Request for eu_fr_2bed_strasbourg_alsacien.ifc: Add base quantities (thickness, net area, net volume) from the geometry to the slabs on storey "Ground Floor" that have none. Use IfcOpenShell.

First a look at what the model holds.

```python
import ifcopenshell
import ifcopenshell.util.element
import ifcopenshell.util.unit

model = ifcopenshell.open("eu_fr_2bed_strasbourg_alsacien.ifc")
print(model.schema)
for unit_type in ("LENGTHUNIT", "AREAUNIT", "VOLUMEUNIT"):
    print(unit_type, ifcopenshell.util.unit.calculate_unit_scale(model, unit_type))
storey = next(s for s in model.by_type("IfcBuildingStorey") if s.Name == "Ground Floor")
slabs = [e for e in ifcopenshell.util.element.get_decomposition(storey) if e.is_a("IfcSlab")]
for e in sorted(slabs, key=lambda e: e.id()):
    print(e.id(), e.is_a(), e.Name, list(ifcopenshell.util.element.get_psets(e, qtos_only=True)), sep=" | ")
```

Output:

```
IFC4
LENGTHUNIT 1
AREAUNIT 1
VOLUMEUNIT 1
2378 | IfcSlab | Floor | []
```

```python
import ifcopenshell
import ifcopenshell.api.pset
import ifcopenshell.geom
import ifcopenshell.util.element
import ifcopenshell.util.shape
import ifcopenshell.util.unit

model = ifcopenshell.open("eu_fr_2bed_strasbourg_alsacien.ifc")
unit_scale = ifcopenshell.util.unit.calculate_unit_scale(model)
area_scale = ifcopenshell.util.unit.calculate_unit_scale(model, "AREAUNIT")
volume_scale = ifcopenshell.util.unit.calculate_unit_scale(model, "VOLUMEUNIT")
settings = ifcopenshell.geom.settings()

storey = next(s for s in model.by_type("IfcBuildingStorey") if s.Name == "Ground Floor")
slabs = [e for e in ifcopenshell.util.element.get_decomposition(storey) if e.is_a("IfcSlab")]

for e in sorted(slabs, key=lambda e: e.id()):
    if ifcopenshell.util.element.get_psets(e, qtos_only=True, should_inherit=False):
        continue
    # Geometry comes back in metres, in the element's own axes.
    shape = ifcopenshell.geom.create_shape(settings, e)
    values = {
        "Width": ifcopenshell.util.shape.get_z(shape.geometry) / unit_scale,
        "NetArea": ifcopenshell.util.shape.get_footprint_area(shape.geometry) / area_scale,
        "NetVolume": ifcopenshell.util.shape.get_volume(shape.geometry) / volume_scale,
    }
    qto = ifcopenshell.api.pset.add_qto(model, product=e, name="Qto_SlabBaseQuantities")
    ifcopenshell.api.pset.edit_qto(model, qto=qto, properties=values)
    print(e.id(), {k: round(v, 3) for k, v in values.items()})

model.write("eu_fr_2bed_strasbourg_alsacien_updated.ifc")
```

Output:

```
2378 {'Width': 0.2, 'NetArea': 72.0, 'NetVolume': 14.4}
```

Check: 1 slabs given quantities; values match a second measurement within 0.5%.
